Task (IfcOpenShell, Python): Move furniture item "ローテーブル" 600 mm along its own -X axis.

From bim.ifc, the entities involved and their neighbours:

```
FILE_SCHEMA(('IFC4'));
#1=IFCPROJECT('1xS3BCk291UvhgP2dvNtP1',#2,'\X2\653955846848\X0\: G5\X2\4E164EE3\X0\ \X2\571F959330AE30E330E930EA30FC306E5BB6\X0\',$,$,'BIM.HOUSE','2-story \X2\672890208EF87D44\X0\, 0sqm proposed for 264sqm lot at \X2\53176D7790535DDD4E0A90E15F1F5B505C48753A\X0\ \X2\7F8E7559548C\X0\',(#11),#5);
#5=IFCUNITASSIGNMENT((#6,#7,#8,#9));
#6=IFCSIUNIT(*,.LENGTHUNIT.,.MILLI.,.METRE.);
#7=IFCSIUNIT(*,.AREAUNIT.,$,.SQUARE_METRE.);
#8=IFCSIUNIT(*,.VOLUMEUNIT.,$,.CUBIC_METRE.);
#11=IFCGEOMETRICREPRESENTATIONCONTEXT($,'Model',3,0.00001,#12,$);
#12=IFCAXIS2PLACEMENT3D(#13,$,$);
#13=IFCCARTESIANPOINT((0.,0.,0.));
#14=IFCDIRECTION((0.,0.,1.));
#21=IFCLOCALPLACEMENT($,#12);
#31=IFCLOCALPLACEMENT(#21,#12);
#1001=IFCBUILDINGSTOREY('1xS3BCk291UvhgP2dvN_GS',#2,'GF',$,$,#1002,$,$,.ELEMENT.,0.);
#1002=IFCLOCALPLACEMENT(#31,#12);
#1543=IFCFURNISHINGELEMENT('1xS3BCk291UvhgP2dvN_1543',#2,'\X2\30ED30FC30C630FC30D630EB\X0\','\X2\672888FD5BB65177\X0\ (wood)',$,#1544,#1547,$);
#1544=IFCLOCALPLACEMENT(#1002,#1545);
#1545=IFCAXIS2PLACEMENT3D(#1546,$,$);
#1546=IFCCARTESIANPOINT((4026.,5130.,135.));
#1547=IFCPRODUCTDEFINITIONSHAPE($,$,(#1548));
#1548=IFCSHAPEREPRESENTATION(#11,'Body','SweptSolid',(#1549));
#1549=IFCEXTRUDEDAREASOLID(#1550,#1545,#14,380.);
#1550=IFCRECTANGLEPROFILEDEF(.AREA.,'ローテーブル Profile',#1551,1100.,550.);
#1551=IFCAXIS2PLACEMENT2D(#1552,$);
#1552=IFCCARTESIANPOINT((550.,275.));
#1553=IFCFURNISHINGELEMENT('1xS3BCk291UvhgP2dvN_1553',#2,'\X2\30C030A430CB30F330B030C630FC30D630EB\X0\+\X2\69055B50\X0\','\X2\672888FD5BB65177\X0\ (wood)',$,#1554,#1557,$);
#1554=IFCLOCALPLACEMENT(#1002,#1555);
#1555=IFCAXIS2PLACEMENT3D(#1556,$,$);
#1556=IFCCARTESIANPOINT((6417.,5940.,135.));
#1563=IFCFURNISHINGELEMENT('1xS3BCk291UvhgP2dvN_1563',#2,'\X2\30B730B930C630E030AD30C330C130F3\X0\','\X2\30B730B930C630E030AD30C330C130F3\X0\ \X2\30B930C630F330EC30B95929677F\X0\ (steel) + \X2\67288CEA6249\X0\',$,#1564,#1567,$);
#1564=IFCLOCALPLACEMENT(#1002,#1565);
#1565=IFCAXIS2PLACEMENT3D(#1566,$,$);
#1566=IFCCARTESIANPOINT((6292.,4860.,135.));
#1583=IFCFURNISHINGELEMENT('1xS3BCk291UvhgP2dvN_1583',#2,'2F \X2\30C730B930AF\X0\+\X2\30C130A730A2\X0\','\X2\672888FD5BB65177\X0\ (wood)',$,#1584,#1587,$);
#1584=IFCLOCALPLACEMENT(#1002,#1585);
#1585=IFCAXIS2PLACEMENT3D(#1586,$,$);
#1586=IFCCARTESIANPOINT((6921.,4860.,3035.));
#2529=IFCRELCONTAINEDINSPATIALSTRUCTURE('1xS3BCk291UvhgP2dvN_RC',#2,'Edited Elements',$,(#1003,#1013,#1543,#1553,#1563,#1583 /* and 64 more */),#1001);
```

```python
import ifcopenshell
import ifcopenshell.api.geometry
import ifcopenshell.util.placement
import ifcopenshell.util.unit

model = ifcopenshell.open("bim.ifc")
unit_scale = ifcopenshell.util.unit.calculate_unit_scale(model)

item = model.by_id(1543)
matrix = ifcopenshell.util.placement.get_local_placement(item.ObjectPlacement)
matrix[:3, 3] -= matrix[:3, 0] * 0.6 / unit_scale
ifcopenshell.api.geometry.edit_object_placement(model, product=item, matrix=matrix, is_si=False)

print(ifcopenshell.util.placement.get_local_placement(item.ObjectPlacement).round(3) + 0.0)

model.write("bim_rev.ifc")
```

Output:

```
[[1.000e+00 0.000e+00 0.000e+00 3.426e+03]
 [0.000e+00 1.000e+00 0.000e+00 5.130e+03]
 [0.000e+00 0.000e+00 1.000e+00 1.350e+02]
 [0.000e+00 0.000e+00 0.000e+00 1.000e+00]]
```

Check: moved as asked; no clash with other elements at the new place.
